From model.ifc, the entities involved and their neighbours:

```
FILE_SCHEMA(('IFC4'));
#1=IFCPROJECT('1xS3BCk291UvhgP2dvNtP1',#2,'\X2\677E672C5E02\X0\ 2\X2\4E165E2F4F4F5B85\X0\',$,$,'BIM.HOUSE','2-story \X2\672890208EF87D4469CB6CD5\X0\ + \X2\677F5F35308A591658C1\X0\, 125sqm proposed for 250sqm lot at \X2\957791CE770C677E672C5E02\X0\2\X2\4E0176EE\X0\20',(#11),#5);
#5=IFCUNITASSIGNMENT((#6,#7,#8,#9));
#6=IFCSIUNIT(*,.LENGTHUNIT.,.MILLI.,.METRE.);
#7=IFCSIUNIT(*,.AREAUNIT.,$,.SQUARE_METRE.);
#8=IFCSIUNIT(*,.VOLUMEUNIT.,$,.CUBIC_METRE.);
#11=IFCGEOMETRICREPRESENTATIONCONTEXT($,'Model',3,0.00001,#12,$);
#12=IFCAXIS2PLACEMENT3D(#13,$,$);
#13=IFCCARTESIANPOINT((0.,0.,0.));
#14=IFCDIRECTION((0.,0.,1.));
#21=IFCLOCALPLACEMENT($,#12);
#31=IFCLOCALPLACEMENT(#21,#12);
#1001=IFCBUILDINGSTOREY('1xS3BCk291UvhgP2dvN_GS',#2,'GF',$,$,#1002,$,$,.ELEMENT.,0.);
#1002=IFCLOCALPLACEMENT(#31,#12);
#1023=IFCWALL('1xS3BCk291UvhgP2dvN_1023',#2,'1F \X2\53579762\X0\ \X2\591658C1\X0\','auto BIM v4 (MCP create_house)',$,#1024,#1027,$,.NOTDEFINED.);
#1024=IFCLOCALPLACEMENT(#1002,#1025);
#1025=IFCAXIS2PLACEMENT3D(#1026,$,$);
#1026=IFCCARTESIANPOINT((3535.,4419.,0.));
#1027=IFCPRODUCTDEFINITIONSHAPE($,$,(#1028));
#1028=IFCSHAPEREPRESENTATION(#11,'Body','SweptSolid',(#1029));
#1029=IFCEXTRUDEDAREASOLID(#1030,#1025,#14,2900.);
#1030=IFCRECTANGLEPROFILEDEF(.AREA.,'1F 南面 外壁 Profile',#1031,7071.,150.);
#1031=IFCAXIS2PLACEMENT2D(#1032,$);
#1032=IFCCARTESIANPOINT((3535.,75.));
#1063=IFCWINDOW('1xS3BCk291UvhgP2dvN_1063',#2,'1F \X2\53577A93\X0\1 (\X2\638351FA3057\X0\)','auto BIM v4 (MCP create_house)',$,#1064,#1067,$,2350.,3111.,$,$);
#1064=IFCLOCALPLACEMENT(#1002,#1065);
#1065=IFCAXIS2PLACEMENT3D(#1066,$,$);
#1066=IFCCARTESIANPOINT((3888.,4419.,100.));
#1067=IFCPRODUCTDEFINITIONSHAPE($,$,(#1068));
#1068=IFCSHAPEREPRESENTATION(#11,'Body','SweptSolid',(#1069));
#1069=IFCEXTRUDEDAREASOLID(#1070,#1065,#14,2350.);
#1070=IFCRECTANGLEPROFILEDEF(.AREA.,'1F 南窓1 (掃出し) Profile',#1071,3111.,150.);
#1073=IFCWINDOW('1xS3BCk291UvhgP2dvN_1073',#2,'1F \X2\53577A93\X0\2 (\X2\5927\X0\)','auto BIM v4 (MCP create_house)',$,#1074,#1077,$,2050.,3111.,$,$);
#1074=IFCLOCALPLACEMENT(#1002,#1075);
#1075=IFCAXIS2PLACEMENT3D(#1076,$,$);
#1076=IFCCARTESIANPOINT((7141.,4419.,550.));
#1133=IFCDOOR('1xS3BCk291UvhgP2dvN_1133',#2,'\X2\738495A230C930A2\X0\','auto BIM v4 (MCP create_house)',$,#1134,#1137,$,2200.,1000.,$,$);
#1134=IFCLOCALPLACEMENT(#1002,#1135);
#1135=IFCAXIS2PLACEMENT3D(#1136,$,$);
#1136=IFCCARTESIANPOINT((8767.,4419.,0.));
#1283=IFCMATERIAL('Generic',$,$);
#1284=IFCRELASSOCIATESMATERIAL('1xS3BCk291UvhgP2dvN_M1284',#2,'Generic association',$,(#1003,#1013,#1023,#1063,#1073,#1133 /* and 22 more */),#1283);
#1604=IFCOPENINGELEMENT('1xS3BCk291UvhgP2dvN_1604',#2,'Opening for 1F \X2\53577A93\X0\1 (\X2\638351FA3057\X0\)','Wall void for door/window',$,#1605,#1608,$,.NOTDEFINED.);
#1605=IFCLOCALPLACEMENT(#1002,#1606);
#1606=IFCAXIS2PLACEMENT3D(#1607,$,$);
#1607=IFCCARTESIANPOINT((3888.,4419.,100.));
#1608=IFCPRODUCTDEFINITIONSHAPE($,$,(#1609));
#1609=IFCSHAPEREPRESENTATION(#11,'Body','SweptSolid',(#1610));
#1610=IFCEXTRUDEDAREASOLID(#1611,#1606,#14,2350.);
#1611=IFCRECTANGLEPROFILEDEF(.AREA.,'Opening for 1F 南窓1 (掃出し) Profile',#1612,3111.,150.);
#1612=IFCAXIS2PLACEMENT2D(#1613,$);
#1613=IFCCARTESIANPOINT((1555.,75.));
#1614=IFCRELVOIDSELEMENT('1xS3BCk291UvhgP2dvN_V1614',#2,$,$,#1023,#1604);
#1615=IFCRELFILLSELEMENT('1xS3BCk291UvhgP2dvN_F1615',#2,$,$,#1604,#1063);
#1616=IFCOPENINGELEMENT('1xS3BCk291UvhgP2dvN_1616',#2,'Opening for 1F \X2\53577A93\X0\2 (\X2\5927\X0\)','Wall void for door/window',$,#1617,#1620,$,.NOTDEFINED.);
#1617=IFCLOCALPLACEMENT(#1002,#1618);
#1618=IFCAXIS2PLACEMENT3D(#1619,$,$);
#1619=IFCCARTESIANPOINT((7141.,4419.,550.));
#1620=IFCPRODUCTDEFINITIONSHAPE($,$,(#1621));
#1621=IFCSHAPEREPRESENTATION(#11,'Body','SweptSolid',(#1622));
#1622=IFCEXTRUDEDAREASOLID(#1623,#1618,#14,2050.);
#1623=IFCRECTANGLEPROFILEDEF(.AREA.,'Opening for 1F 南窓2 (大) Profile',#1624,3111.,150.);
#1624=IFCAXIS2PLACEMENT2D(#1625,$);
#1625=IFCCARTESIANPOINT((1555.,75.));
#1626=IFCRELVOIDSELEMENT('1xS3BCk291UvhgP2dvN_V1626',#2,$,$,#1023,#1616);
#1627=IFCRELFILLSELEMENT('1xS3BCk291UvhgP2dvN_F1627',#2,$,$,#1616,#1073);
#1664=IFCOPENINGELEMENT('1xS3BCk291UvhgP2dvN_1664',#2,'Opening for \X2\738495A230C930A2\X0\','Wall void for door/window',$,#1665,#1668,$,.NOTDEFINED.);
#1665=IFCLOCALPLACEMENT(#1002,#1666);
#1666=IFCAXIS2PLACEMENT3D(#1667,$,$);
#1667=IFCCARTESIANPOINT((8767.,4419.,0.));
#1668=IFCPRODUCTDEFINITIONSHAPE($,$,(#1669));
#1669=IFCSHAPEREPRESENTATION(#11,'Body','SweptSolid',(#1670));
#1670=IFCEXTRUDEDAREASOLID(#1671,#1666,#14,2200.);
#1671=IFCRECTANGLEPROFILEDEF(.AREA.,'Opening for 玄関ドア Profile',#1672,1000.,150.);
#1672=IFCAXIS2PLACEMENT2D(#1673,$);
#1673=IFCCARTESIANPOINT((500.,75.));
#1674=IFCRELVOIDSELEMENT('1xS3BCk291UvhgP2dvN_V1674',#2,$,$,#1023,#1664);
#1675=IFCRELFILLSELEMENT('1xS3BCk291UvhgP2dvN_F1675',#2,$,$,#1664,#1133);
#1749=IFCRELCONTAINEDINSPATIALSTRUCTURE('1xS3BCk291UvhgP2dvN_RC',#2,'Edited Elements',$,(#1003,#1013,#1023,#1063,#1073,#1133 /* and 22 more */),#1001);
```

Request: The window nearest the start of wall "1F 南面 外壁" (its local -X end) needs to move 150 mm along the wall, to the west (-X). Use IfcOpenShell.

```python
import ifcopenshell
import ifcopenshell.api.geometry
import ifcopenshell.util.placement

model = ifcopenshell.open("model.ifc")

window = model.by_guid("1xS3BCk291UvhgP2dvN_1063")
opening = window.FillsVoids[0].RelatingOpeningElement
wall = opening.VoidsElements[0].RelatingBuildingElement

wall_matrix = ifcopenshell.util.placement.get_local_placement(wall.ObjectPlacement)
shift = wall_matrix[:3, 0] * -150.0
before = ifcopenshell.util.placement.get_local_placement(window.ObjectPlacement)[:3, 3].copy()

# The window is not placed relative to its opening, so move both.
for product in (opening, window):
    matrix = ifcopenshell.util.placement.get_local_placement(product.ObjectPlacement)
    matrix[:3, 3] += shift
    ifcopenshell.api.geometry.edit_object_placement(model, product=product, matrix=matrix, is_si=False)

after = ifcopenshell.util.placement.get_local_placement(window.ObjectPlacement)[:3, 3]
print("window moved by", (after - before).round(3) + 0.0)

model.write("model_edited.ifc")
```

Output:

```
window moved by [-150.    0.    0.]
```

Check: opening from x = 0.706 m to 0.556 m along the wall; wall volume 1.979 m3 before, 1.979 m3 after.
